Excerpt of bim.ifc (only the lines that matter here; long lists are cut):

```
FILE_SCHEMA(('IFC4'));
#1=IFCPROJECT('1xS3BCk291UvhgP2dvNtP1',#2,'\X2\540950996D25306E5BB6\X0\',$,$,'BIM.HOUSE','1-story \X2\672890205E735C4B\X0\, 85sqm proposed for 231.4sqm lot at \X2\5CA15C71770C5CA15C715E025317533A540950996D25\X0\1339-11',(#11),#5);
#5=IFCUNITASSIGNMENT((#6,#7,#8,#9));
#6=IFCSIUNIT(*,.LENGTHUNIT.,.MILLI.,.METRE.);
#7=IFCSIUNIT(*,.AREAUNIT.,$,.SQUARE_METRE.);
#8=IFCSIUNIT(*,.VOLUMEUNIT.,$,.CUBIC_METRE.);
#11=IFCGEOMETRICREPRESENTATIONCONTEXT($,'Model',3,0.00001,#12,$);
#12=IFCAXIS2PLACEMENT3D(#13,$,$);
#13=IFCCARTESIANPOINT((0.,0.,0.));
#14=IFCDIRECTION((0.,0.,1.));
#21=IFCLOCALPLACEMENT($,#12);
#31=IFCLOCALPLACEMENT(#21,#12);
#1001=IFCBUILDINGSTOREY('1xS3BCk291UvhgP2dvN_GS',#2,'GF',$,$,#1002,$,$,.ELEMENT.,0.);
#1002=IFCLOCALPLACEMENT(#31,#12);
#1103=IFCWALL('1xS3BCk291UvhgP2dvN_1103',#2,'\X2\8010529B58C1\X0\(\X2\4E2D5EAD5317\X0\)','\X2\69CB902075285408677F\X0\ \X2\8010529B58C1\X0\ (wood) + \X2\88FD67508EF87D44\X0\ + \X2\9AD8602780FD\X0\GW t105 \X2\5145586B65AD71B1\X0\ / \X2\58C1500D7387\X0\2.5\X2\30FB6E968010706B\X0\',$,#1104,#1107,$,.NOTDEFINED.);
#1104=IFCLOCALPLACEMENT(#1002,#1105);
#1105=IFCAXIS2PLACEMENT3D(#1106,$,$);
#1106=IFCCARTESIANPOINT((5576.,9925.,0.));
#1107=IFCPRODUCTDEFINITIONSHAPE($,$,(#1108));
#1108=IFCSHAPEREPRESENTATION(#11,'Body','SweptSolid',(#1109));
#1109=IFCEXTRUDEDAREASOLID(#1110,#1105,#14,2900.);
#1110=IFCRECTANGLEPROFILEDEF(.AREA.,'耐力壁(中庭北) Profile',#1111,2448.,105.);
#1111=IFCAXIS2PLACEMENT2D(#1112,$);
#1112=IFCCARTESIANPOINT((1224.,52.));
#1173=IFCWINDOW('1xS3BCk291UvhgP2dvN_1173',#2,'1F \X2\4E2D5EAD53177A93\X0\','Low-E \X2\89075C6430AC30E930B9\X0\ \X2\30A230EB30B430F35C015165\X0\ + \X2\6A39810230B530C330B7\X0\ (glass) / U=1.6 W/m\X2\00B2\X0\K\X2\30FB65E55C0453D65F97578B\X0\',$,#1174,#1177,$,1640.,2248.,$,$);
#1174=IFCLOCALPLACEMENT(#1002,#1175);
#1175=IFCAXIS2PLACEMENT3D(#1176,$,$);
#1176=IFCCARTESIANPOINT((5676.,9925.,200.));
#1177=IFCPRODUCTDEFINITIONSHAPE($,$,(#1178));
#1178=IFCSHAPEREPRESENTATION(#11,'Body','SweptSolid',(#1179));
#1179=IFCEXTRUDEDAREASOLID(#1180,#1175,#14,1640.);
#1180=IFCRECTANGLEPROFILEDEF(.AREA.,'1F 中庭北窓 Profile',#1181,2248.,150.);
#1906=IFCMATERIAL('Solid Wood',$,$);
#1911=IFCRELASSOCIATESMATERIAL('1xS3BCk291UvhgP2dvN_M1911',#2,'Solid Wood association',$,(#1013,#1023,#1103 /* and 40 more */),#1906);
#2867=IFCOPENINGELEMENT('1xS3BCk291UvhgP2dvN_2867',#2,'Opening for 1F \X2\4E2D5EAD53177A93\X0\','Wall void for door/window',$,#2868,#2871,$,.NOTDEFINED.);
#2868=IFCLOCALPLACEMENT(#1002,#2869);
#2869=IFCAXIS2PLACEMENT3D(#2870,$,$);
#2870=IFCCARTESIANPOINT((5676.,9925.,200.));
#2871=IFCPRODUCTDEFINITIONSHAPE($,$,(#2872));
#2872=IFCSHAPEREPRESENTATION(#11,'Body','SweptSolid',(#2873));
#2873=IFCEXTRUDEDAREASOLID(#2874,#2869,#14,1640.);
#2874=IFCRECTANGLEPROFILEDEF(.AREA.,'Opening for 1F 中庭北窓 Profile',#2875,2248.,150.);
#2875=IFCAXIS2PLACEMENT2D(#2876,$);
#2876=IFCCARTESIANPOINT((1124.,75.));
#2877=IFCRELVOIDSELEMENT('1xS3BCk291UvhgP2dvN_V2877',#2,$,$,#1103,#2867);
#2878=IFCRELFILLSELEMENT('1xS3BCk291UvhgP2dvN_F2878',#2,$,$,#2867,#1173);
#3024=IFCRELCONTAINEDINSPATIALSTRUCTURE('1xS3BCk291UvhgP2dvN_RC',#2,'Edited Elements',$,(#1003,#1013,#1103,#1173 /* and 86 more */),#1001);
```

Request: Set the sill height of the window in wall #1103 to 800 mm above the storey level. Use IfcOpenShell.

```python
import numpy as np
import ifcopenshell
import ifcopenshell.api.geometry
import ifcopenshell.geom
import ifcopenshell.util.element
import ifcopenshell.util.placement
import ifcopenshell.util.shape
import ifcopenshell.util.unit

model = ifcopenshell.open("bim.ifc")
unit_scale = ifcopenshell.util.unit.calculate_unit_scale(model)

window = model.by_guid("1xS3BCk291UvhgP2dvN_1173")
opening = window.FillsVoids[0].RelatingOpeningElement
storey = ifcopenshell.util.element.get_container(window, ifc_class="IfcBuildingStorey")
level = ifcopenshell.util.placement.get_local_placement(storey.ObjectPlacement)[2, 3]

# The opening's origin need not be at the sill, so measure its lowest point.
shape = ifcopenshell.geom.create_shape(ifcopenshell.geom.settings(), opening)
bottom = ifcopenshell.util.shape.get_shape_bottom_elevation(shape, shape.geometry) / unit_scale
dz = level + 0.8 / unit_scale - bottom

shift = np.array([0.0, 0.0, dz])
# The window is not placed relative to its opening, so move both.
for product in (opening, window):
    matrix = ifcopenshell.util.placement.get_local_placement(product.ObjectPlacement)
    matrix[:3, 3] += shift
    ifcopenshell.api.geometry.edit_object_placement(model, product=product, matrix=matrix, is_si=False)

print(f"moved by {dz * unit_scale:+.3f} m")

model.write("bim_rev.ifc")
```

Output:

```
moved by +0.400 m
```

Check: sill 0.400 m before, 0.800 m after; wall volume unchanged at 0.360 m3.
